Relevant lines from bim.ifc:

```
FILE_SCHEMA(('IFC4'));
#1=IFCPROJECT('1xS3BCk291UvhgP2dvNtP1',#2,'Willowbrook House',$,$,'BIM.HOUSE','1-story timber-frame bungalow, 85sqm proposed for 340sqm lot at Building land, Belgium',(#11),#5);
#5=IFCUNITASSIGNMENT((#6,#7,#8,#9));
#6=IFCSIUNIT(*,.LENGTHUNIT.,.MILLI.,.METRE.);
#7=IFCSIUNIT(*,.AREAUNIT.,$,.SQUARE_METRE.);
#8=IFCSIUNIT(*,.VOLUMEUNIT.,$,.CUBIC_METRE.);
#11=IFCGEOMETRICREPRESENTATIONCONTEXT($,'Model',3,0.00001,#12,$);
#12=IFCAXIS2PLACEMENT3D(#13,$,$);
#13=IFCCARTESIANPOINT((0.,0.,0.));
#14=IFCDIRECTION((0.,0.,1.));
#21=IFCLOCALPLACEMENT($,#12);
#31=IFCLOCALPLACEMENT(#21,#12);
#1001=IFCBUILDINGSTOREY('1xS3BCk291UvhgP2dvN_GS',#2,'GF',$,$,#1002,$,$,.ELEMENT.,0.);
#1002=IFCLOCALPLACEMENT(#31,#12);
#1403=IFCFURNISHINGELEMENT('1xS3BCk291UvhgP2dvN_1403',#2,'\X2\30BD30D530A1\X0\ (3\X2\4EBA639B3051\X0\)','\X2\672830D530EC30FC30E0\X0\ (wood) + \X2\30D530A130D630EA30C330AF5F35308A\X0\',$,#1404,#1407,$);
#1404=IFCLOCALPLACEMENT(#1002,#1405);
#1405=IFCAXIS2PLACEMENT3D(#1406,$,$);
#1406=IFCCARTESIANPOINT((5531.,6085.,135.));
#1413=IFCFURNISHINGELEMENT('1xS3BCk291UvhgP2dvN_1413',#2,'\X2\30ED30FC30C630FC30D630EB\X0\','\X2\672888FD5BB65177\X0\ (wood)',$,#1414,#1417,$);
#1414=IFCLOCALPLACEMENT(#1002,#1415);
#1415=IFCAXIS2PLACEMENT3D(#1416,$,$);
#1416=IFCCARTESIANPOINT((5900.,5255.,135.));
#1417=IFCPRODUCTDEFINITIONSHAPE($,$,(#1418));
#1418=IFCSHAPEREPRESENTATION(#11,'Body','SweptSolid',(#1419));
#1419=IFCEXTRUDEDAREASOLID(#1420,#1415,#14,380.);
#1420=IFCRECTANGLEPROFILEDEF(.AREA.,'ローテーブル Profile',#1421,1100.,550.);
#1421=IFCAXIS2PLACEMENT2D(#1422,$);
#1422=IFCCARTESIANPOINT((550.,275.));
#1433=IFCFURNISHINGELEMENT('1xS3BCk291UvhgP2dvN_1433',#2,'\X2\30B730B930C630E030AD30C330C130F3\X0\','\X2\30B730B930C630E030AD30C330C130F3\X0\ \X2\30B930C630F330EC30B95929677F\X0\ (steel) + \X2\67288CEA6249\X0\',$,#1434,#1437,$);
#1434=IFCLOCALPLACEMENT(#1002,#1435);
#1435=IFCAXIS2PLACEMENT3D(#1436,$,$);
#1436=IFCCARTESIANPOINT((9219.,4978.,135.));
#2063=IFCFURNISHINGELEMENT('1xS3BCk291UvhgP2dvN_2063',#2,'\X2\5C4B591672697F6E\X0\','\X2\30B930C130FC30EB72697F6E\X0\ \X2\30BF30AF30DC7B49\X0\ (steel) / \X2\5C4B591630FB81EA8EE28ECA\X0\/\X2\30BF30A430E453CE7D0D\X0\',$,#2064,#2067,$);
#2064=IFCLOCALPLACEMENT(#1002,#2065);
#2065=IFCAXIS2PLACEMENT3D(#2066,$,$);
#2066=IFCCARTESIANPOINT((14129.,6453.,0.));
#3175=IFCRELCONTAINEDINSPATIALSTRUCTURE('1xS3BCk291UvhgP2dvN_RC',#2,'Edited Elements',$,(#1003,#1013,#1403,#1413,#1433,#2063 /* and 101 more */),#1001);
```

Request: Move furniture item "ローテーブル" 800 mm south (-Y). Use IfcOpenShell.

```python
import ifcopenshell
import ifcopenshell.api.geometry
import ifcopenshell.util.placement

model = ifcopenshell.open("bim.ifc")

item = model.by_guid("1xS3BCk291UvhgP2dvN_1413")
matrix = ifcopenshell.util.placement.get_local_placement(item.ObjectPlacement)
matrix[1, 3] -= 800.0
ifcopenshell.api.geometry.edit_object_placement(model, product=item, matrix=matrix, is_si=False)

print(ifcopenshell.util.placement.get_local_placement(item.ObjectPlacement).round(3) + 0.0)

model.write("bim-out.ifc")
```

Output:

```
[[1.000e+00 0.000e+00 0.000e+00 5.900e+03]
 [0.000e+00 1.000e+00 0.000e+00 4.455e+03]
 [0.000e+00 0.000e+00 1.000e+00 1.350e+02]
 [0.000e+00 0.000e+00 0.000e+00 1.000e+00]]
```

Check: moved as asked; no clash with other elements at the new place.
